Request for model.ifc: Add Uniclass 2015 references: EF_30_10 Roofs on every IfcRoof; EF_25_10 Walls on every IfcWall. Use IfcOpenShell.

First a look at what the model holds.

```python
import ifcopenshell

model = ifcopenshell.open("model.ifc")
print(model.schema)
print("classifications:", [c.Name for c in model.by_type("IfcClassification")])
for ifc_class in ("IfcDoor", "IfcRoof", "IfcStair", "IfcWall", "IfcWindow"):
    print(ifc_class, len(model.by_type(ifc_class)))
```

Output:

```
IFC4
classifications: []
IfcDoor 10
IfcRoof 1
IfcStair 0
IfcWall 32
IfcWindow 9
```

```python
import ifcopenshell
import ifcopenshell.api.classification

model = ifcopenshell.open("model.ifc")

system = ifcopenshell.api.classification.add_classification(model, classification="Uniclass 2015")

codes = {
    "IfcRoof": ("EF_30_10", "Roofs"),
    "IfcWall": ("EF_25_10", "Walls"),
}
for ifc_class, (code, name) in codes.items():
    products = model.by_type(ifc_class)
    ifcopenshell.api.classification.add_reference(
        model, products=products, classification=system, identification=code, name=name
    )
    print(code, len(products))

model.write("model_updated.ifc")
```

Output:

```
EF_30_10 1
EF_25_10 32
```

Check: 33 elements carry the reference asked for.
